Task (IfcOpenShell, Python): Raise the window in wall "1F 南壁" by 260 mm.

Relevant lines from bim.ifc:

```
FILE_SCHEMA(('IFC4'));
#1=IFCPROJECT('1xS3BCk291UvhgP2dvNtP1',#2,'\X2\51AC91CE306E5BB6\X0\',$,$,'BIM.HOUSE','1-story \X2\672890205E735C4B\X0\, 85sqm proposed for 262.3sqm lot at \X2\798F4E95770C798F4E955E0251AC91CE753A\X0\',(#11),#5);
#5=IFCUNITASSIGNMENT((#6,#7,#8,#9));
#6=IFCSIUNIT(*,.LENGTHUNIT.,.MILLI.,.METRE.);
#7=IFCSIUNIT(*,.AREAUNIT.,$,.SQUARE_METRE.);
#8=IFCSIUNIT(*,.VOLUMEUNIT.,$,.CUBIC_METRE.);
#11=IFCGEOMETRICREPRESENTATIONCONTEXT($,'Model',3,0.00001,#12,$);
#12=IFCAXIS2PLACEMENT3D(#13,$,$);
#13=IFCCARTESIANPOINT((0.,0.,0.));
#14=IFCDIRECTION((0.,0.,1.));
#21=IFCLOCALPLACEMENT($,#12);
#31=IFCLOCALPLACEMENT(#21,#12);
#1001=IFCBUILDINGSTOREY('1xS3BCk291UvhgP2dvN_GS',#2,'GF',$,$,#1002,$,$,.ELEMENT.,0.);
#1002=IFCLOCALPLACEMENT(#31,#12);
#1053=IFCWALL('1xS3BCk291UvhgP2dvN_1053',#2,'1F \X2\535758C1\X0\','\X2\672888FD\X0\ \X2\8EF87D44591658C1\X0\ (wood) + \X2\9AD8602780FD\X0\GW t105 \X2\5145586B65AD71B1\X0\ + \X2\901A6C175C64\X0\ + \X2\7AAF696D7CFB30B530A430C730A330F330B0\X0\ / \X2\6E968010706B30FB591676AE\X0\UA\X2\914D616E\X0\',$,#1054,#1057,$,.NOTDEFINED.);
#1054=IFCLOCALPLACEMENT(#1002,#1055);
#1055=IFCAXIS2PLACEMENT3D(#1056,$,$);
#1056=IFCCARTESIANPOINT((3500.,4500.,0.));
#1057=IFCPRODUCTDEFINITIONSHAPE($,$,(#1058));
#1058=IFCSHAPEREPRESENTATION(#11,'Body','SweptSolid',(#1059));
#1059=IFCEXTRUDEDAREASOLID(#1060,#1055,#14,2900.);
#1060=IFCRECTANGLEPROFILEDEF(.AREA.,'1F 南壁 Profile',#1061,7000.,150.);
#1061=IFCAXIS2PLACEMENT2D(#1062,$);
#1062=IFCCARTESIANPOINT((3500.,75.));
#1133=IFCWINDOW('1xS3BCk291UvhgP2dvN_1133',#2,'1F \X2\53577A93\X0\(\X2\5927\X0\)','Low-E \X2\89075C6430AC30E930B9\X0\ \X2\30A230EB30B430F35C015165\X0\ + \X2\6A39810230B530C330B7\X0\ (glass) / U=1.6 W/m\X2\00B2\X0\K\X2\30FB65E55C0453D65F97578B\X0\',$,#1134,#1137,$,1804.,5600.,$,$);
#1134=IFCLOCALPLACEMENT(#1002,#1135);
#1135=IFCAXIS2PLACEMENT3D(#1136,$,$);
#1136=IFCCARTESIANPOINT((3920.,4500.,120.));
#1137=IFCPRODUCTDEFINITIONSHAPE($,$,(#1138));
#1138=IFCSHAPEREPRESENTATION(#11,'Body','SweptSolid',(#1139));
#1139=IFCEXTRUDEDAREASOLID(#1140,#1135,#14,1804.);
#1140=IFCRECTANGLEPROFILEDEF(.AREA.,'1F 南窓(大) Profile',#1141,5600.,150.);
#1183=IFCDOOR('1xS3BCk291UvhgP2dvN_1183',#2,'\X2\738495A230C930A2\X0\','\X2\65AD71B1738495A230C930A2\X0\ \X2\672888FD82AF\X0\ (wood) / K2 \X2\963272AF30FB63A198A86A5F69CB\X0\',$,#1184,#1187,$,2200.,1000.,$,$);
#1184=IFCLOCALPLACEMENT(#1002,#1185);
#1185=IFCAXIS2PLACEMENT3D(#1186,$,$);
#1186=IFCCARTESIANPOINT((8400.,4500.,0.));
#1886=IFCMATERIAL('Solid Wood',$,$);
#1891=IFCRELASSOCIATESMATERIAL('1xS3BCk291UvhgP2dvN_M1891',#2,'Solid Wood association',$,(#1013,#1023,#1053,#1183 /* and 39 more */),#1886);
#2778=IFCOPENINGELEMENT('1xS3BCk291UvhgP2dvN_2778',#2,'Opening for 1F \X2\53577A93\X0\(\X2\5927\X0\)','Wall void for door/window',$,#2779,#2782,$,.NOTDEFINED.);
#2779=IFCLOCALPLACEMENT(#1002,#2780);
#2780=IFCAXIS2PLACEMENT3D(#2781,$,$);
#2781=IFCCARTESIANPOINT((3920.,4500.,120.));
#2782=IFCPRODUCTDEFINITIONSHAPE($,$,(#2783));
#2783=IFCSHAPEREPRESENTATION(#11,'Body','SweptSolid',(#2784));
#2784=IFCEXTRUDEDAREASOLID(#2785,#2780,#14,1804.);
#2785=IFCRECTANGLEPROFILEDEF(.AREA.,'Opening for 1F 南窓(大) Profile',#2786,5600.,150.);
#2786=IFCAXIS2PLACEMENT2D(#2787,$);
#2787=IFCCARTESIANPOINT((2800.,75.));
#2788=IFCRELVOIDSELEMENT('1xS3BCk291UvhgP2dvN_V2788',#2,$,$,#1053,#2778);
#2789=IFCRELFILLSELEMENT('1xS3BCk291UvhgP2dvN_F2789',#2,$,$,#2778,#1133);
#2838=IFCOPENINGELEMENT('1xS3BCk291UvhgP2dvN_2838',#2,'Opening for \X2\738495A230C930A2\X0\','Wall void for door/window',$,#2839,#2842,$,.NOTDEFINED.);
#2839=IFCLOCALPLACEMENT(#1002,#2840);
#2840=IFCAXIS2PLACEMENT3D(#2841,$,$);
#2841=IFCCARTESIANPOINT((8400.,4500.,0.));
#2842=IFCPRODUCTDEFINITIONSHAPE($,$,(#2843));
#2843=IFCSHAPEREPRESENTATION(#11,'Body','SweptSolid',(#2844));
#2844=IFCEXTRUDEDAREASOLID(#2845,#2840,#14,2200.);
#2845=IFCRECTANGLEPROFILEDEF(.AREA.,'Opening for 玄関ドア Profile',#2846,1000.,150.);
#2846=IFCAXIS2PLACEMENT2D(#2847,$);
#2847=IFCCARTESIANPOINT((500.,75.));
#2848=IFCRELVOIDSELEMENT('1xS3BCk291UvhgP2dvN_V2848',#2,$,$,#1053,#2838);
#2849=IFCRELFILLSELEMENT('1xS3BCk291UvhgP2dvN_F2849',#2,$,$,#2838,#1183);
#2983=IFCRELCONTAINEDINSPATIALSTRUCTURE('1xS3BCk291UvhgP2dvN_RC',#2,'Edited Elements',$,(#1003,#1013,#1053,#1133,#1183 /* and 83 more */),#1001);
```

```python
import numpy as np
import ifcopenshell
import ifcopenshell.api.geometry
import ifcopenshell.util.placement
import ifcopenshell.util.unit

model = ifcopenshell.open("bim.ifc")
unit_scale = ifcopenshell.util.unit.calculate_unit_scale(model)

window = model.by_guid("1xS3BCk291UvhgP2dvN_1133")
opening = window.FillsVoids[0].RelatingOpeningElement
dz = 0.26 / unit_scale

shift = np.array([0.0, 0.0, dz])
# The window is not placed relative to its opening, so move both.
for product in (opening, window):
    matrix = ifcopenshell.util.placement.get_local_placement(product.ObjectPlacement)
    matrix[:3, 3] += shift
    ifcopenshell.api.geometry.edit_object_placement(model, product=product, matrix=matrix, is_si=False)

print(f"moved by {dz * unit_scale:+.3f} m")

model.write("bim_updated.ifc")
```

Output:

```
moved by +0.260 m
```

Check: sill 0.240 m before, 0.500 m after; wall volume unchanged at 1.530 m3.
